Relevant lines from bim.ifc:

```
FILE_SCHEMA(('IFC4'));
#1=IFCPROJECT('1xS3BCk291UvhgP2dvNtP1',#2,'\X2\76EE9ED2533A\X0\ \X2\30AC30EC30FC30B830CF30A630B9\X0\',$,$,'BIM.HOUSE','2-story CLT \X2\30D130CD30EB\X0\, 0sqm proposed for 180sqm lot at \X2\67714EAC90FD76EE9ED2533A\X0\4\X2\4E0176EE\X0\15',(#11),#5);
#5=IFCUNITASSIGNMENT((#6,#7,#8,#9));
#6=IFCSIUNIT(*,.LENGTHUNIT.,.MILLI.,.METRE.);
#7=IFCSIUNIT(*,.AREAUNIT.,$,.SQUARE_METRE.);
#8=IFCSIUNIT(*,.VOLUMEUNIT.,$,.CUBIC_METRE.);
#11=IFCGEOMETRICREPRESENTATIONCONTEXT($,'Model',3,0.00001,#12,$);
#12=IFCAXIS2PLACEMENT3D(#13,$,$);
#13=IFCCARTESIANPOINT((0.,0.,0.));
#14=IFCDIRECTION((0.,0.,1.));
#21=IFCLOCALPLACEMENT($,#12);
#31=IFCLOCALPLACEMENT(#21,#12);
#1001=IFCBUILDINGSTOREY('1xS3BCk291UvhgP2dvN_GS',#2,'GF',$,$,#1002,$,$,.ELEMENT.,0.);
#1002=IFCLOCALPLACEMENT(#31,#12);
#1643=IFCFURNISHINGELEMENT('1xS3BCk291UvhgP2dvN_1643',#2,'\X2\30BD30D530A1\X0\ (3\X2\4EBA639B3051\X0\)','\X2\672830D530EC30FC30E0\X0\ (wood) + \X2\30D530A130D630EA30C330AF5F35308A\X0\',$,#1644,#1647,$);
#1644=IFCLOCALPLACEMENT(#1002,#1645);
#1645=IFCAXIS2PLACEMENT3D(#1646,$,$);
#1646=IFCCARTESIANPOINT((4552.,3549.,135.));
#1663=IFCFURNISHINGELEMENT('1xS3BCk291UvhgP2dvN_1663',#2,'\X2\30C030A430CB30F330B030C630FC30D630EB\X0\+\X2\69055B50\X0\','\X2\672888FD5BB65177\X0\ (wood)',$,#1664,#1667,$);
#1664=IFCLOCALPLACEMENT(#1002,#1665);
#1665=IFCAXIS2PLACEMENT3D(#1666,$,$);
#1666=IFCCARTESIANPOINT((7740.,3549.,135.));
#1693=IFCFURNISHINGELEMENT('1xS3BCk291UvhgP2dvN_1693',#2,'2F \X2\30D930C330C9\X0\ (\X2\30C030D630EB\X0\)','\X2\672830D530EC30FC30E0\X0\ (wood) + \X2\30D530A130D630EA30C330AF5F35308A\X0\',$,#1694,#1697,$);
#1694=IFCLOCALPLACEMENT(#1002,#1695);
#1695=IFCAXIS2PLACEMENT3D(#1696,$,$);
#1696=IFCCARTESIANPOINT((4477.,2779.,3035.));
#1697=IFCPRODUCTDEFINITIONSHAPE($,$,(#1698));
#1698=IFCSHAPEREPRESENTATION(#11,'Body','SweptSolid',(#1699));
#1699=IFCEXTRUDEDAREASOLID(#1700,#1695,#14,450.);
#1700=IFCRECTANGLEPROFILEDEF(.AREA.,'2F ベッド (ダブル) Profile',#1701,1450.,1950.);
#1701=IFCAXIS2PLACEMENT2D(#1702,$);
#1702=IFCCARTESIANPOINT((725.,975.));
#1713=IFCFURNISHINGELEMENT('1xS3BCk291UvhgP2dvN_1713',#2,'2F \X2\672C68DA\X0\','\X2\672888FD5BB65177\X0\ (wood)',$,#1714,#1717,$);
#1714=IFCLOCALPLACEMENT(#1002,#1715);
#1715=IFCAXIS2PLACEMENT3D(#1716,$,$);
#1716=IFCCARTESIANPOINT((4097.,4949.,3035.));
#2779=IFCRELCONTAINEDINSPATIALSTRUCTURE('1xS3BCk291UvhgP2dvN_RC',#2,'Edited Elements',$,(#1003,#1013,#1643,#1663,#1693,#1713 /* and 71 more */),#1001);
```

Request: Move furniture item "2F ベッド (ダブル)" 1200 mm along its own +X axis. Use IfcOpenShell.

```python
import ifcopenshell
import ifcopenshell.api.geometry
import ifcopenshell.util.placement

model = ifcopenshell.open("bim.ifc")

item = model.by_id(1693)
matrix = ifcopenshell.util.placement.get_local_placement(item.ObjectPlacement)
matrix[:3, 3] += matrix[:3, 0] * 1200.0
ifcopenshell.api.geometry.edit_object_placement(model, product=item, matrix=matrix, is_si=False)

print(ifcopenshell.util.placement.get_local_placement(item.ObjectPlacement).round(3) + 0.0)

model.write("bim_rev.ifc")
```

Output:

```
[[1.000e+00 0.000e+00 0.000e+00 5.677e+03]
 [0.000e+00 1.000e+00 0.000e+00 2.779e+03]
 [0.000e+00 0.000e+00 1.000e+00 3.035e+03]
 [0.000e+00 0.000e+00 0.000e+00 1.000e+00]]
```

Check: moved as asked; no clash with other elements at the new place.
